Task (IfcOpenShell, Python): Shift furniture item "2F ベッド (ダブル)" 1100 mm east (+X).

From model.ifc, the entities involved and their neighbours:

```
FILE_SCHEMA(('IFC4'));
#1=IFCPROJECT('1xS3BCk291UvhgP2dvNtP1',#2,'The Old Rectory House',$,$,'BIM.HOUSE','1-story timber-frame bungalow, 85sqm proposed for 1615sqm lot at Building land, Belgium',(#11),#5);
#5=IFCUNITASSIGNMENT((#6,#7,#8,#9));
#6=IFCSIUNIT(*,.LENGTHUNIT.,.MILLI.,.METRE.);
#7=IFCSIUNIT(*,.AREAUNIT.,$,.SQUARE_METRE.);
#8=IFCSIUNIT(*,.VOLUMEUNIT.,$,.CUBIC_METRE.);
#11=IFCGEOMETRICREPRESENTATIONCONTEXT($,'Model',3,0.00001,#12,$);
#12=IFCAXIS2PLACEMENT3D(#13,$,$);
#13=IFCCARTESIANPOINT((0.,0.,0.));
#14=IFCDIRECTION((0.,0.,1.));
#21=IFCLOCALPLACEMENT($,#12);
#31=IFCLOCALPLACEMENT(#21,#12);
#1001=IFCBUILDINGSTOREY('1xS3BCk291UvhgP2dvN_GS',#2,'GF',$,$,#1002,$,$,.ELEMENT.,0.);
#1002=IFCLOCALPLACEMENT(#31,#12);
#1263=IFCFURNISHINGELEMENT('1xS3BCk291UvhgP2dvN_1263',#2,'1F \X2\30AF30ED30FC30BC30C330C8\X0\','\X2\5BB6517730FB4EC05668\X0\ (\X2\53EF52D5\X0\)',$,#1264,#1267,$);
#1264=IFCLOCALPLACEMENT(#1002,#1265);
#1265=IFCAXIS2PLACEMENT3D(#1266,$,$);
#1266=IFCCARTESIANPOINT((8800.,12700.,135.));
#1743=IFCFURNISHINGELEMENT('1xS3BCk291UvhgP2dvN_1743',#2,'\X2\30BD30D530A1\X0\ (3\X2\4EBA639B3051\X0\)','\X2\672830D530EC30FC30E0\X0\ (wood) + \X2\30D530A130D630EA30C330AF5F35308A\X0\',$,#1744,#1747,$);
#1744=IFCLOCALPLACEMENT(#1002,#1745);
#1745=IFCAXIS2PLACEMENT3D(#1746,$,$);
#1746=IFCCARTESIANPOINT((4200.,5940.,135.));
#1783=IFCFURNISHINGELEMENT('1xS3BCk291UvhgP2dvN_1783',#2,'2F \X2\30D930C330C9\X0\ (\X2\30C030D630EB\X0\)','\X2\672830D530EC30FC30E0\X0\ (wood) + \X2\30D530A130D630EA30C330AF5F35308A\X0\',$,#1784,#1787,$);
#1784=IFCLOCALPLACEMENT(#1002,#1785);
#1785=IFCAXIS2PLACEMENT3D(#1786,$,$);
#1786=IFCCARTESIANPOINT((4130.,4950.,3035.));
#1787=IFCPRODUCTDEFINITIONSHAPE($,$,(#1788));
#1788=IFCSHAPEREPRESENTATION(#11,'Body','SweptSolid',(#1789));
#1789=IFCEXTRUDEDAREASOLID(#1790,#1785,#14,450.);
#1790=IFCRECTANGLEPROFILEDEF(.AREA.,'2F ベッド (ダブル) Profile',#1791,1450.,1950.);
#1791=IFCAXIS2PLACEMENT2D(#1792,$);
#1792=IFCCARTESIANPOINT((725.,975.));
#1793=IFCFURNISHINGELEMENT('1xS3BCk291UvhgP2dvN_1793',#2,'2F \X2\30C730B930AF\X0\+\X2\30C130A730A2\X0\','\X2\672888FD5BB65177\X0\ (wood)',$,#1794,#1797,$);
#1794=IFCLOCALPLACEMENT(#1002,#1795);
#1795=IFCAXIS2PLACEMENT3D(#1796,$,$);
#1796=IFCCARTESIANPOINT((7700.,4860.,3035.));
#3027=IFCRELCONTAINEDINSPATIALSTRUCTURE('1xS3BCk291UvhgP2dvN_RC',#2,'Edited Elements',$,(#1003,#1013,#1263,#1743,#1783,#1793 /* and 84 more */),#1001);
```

```python
import ifcopenshell
import ifcopenshell.api.geometry
import ifcopenshell.util.placement
import ifcopenshell.util.unit

model = ifcopenshell.open("model.ifc")
unit_scale = ifcopenshell.util.unit.calculate_unit_scale(model)

item = model.by_guid("1xS3BCk291UvhgP2dvN_1783")
matrix = ifcopenshell.util.placement.get_local_placement(item.ObjectPlacement)
matrix[0, 3] += 1.1 / unit_scale
ifcopenshell.api.geometry.edit_object_placement(model, product=item, matrix=matrix, is_si=False)

print(ifcopenshell.util.placement.get_local_placement(item.ObjectPlacement).round(3) + 0.0)

model.write("model_updated.ifc")
```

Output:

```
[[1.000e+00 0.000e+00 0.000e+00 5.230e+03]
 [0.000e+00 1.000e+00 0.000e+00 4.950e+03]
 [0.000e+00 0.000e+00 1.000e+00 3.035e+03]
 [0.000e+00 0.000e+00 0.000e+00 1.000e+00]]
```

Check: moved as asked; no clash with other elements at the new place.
